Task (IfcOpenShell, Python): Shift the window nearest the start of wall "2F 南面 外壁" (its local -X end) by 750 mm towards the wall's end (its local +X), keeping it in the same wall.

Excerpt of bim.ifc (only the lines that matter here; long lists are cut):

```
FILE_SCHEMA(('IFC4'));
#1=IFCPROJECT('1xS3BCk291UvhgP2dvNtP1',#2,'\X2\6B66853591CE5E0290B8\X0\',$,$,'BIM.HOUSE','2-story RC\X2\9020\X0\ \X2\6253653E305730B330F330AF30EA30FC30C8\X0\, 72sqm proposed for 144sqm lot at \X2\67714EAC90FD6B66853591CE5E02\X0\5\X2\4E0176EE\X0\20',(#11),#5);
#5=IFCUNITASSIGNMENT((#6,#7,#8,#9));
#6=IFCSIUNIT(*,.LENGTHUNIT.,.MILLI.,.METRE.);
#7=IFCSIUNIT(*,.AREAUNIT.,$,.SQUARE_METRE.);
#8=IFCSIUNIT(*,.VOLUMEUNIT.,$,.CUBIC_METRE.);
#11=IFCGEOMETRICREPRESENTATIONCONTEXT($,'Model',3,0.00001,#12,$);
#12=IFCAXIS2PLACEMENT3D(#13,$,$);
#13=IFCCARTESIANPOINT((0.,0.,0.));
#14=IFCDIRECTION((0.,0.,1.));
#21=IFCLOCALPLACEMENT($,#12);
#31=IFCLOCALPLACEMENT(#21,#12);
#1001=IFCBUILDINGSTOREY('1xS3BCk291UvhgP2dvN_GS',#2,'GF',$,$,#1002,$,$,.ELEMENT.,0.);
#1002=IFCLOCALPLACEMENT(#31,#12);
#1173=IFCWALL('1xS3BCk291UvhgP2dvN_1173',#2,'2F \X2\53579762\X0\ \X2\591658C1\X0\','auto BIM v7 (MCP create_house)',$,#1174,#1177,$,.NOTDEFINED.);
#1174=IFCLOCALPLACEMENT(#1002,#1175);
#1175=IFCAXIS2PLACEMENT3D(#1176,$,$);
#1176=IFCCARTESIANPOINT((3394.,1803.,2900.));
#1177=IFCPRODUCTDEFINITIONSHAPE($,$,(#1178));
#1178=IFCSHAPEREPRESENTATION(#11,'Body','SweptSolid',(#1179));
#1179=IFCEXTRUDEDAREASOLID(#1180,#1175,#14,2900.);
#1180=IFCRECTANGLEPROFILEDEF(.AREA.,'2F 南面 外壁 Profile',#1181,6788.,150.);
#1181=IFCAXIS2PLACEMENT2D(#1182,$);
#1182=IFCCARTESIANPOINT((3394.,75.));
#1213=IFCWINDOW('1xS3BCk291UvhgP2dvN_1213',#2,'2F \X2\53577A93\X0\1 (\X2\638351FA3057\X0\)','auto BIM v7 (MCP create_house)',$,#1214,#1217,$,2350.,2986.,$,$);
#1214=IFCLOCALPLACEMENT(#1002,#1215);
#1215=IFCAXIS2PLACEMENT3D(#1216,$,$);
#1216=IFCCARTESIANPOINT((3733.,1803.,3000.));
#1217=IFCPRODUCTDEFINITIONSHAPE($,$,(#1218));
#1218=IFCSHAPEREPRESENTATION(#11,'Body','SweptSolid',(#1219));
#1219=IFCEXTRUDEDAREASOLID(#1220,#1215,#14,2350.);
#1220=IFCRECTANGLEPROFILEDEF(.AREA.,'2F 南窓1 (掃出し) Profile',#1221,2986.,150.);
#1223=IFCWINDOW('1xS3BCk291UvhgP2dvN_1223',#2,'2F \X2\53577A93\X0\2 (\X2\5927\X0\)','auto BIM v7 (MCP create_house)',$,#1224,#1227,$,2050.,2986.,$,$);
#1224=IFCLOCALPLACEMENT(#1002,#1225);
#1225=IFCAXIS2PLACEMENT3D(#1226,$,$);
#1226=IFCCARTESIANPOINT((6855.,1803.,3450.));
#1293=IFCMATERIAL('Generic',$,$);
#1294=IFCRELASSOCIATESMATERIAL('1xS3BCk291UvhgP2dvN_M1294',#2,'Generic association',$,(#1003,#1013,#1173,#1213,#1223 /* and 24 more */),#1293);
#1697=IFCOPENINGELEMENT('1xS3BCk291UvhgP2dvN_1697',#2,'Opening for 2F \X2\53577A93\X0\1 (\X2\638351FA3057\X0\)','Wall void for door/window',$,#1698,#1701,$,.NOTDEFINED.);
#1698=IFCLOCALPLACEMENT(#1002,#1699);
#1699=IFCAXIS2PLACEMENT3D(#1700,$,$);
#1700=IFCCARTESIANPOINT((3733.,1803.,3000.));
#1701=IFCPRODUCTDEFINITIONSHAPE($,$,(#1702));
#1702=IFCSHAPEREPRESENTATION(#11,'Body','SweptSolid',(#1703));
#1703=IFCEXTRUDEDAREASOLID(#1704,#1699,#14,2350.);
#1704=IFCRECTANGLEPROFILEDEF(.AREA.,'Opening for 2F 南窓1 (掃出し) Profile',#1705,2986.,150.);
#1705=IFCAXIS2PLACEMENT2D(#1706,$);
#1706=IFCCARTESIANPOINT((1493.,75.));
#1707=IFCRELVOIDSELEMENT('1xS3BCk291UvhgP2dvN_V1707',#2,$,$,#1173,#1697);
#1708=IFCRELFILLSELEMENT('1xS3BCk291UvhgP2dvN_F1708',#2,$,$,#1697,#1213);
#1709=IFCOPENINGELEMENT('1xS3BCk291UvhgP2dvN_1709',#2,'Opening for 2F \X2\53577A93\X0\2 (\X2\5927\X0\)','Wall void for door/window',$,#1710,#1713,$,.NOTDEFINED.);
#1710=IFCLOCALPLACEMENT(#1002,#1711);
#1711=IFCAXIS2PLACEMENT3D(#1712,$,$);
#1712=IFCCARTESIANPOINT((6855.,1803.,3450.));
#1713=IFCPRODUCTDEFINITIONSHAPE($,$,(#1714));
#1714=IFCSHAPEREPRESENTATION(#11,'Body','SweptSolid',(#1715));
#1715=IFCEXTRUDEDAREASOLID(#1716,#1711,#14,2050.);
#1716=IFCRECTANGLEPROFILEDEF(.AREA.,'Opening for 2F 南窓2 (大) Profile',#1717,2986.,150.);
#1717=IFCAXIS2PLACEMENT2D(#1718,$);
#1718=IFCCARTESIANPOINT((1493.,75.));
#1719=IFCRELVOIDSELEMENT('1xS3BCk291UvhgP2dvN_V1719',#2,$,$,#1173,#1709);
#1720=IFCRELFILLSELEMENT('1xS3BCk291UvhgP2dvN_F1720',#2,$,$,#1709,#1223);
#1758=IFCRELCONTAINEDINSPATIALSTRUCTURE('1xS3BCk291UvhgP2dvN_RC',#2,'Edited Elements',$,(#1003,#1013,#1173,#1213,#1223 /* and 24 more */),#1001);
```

```python
import ifcopenshell
import ifcopenshell.api.geometry
import ifcopenshell.util.placement
import ifcopenshell.util.unit

model = ifcopenshell.open("bim.ifc")
unit_scale = ifcopenshell.util.unit.calculate_unit_scale(model)

window = model.by_guid("1xS3BCk291UvhgP2dvN_1213")
opening = window.FillsVoids[0].RelatingOpeningElement
wall = opening.VoidsElements[0].RelatingBuildingElement

wall_matrix = ifcopenshell.util.placement.get_local_placement(wall.ObjectPlacement)
shift = wall_matrix[:3, 0] * 0.75 / unit_scale
before = ifcopenshell.util.placement.get_local_placement(window.ObjectPlacement)[:3, 3].copy()

# The window is not placed relative to its opening, so move both.
for product in (opening, window):
    matrix = ifcopenshell.util.placement.get_local_placement(product.ObjectPlacement)
    matrix[:3, 3] += shift
    ifcopenshell.api.geometry.edit_object_placement(model, product=product, matrix=matrix, is_si=False)

after = ifcopenshell.util.placement.get_local_placement(window.ObjectPlacement)[:3, 3]
print("window moved by", (after - before).round(3) + 0.0)

model.write("bim_v2.ifc")
```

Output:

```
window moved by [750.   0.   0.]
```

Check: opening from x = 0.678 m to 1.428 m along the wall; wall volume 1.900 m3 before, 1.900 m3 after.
